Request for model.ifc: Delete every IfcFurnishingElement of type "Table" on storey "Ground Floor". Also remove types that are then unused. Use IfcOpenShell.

First a look at what the model holds.

```python
import ifcopenshell
import ifcopenshell.util.element

model = ifcopenshell.open("model.ifc")
print(model.schema)
storey = next(s for s in model.by_type("IfcBuildingStorey") if s.Name == "Ground Floor")
furniture = [e for e in ifcopenshell.util.element.get_decomposition(storey) if e.is_a("IfcFurnishingElement")]
seen = {}
for e in furniture:
    element_type = ifcopenshell.util.element.get_type(e)
    name = element_type.Name if element_type not in (None, e) else None
    seen[name] = seen.get(name, 0) + 1
for name, count in sorted(seen.items(), key=str):
    print(count, "x", name)
```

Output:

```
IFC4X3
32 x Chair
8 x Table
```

```python
import ifcopenshell
import ifcopenshell.api.root
import ifcopenshell.util.element

model = ifcopenshell.open("model.ifc")

storey = next(s for s in model.by_type("IfcBuildingStorey") if s.Name == "Ground Floor")
furniture = [e for e in ifcopenshell.util.element.get_decomposition(storey) if e.is_a("IfcFurnishingElement")]
targets = [e for e in furniture if (t := ifcopenshell.util.element.get_type(e)) not in (None, e) and t.Name == "Table"]
types = {ifcopenshell.util.element.get_type(e) for e in targets} - {None, *targets}

for e in targets:
    ifcopenshell.api.root.remove_product(model, product=e)
print(len(targets), "removed")

unused = [t for t in types if not ifcopenshell.util.element.get_types(t)]
for t in unused:
    ifcopenshell.api.root.remove_product(model, product=t)
print(len(unused), "unused types removed")

model.write("model_updated.ifc")
```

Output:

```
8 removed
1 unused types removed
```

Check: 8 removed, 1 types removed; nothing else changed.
